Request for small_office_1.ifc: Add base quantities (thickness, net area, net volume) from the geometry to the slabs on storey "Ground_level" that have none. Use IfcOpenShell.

First a look at what the model holds.

```python
import ifcopenshell
import ifcopenshell.util.element
import ifcopenshell.util.unit

model = ifcopenshell.open("small_office_1.ifc")
print(model.schema)
for unit_type in ("LENGTHUNIT", "AREAUNIT", "VOLUMEUNIT"):
    print(unit_type, ifcopenshell.util.unit.calculate_unit_scale(model, unit_type))
storey = next(s for s in model.by_type("IfcBuildingStorey") if s.Name == "Ground_level")
slabs = [e for e in ifcopenshell.util.element.get_decomposition(storey) if e.is_a("IfcSlab")]
for e in sorted(slabs, key=lambda e: e.id()):
    print(e.id(), e.is_a(), e.Name, list(ifcopenshell.util.element.get_psets(e, qtos_only=True)), sep=" | ")
```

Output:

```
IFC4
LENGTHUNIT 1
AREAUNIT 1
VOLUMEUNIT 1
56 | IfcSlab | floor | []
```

```python
import ifcopenshell
import ifcopenshell.api.pset
import ifcopenshell.geom
import ifcopenshell.util.element
import ifcopenshell.util.shape
import ifcopenshell.util.unit

model = ifcopenshell.open("small_office_1.ifc")
unit_scale = ifcopenshell.util.unit.calculate_unit_scale(model)
area_scale = ifcopenshell.util.unit.calculate_unit_scale(model, "AREAUNIT")
volume_scale = ifcopenshell.util.unit.calculate_unit_scale(model, "VOLUMEUNIT")
settings = ifcopenshell.geom.settings()

storey = next(s for s in model.by_type("IfcBuildingStorey") if s.Name == "Ground_level")
slabs = [e for e in ifcopenshell.util.element.get_decomposition(storey) if e.is_a("IfcSlab")]

for e in sorted(slabs, key=lambda e: e.id()):
    if ifcopenshell.util.element.get_psets(e, qtos_only=True, should_inherit=False):
        continue
    # Geometry comes back in metres, in the element's own axes.
    shape = ifcopenshell.geom.create_shape(settings, e)
    values = {
        "Width": ifcopenshell.util.shape.get_z(shape.geometry) / unit_scale,
        "NetArea": ifcopenshell.util.shape.get_footprint_area(shape.geometry) / area_scale,
        "NetVolume": ifcopenshell.util.shape.get_volume(shape.geometry) / volume_scale,
    }
    qto = ifcopenshell.api.pset.add_qto(model, product=e, name="Qto_SlabBaseQuantities")
    ifcopenshell.api.pset.edit_qto(model, qto=qto, properties=values)
    print(e.id(), {k: round(v, 3) for k, v in values.items()})

model.write("small_office_1_updated.ifc")
```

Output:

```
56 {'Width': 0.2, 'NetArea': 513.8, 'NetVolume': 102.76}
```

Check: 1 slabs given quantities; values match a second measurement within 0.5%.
